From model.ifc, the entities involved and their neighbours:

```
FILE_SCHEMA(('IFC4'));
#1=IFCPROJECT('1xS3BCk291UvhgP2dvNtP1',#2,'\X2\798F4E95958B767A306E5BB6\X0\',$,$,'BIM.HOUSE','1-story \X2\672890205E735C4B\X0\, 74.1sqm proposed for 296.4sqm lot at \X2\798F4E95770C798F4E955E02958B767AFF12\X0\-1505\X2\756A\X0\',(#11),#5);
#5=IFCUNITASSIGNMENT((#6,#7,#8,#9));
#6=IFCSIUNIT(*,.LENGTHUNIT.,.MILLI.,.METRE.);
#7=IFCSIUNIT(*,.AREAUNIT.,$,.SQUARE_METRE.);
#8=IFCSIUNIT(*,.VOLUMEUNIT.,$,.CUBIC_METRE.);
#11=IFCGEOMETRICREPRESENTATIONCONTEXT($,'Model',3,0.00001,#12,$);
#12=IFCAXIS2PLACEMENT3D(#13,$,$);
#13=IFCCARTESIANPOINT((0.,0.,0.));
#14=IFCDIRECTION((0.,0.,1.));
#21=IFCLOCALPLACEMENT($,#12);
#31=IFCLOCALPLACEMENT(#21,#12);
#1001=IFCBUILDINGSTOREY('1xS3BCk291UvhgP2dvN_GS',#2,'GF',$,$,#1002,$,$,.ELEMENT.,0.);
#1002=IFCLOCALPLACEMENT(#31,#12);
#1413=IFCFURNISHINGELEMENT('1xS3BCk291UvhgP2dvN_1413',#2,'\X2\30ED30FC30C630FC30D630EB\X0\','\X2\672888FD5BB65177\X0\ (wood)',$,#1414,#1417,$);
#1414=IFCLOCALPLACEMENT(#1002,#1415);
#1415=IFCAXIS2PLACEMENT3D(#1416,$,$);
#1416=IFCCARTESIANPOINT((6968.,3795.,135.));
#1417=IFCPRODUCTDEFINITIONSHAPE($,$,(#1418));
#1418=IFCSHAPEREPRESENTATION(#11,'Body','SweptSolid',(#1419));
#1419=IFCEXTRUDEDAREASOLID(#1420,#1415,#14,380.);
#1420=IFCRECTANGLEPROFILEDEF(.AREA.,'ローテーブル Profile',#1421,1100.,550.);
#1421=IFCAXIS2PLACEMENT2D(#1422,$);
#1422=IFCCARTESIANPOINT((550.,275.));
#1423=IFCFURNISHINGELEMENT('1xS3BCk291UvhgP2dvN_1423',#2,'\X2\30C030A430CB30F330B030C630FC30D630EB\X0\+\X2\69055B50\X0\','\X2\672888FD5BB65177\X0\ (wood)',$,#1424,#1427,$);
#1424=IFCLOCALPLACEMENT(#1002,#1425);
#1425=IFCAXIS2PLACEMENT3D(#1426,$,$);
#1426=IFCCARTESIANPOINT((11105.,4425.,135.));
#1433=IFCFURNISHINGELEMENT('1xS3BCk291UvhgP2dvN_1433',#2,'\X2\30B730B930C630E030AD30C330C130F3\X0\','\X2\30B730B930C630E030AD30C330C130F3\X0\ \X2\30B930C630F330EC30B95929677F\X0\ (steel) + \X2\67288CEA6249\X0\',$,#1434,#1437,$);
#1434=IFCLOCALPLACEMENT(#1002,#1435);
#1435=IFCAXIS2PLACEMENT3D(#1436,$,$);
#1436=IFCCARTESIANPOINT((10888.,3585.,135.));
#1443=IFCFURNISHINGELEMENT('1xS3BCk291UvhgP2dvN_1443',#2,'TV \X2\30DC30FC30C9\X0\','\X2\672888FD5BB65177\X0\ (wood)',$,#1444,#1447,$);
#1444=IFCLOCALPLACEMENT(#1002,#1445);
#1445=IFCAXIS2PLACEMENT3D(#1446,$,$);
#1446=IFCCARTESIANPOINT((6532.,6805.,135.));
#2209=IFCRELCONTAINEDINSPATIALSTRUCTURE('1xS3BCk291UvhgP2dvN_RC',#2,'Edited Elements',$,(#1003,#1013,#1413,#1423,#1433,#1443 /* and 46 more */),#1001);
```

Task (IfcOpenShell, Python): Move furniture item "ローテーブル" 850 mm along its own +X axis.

```python
import ifcopenshell
import ifcopenshell.api.geometry
import ifcopenshell.util.placement
import ifcopenshell.util.unit

model = ifcopenshell.open("model.ifc")
unit_scale = ifcopenshell.util.unit.calculate_unit_scale(model)

item = model.by_guid("1xS3BCk291UvhgP2dvN_1413")
matrix = ifcopenshell.util.placement.get_local_placement(item.ObjectPlacement)
matrix[:3, 3] += matrix[:3, 0] * 0.85 / unit_scale
ifcopenshell.api.geometry.edit_object_placement(model, product=item, matrix=matrix, is_si=False)

print(ifcopenshell.util.placement.get_local_placement(item.ObjectPlacement).round(3) + 0.0)

model.write("model_rev.ifc")
```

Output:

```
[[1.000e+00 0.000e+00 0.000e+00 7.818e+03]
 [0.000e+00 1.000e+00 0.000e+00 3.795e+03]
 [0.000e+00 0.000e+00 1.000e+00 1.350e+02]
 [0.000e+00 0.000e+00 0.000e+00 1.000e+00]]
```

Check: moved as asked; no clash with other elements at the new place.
